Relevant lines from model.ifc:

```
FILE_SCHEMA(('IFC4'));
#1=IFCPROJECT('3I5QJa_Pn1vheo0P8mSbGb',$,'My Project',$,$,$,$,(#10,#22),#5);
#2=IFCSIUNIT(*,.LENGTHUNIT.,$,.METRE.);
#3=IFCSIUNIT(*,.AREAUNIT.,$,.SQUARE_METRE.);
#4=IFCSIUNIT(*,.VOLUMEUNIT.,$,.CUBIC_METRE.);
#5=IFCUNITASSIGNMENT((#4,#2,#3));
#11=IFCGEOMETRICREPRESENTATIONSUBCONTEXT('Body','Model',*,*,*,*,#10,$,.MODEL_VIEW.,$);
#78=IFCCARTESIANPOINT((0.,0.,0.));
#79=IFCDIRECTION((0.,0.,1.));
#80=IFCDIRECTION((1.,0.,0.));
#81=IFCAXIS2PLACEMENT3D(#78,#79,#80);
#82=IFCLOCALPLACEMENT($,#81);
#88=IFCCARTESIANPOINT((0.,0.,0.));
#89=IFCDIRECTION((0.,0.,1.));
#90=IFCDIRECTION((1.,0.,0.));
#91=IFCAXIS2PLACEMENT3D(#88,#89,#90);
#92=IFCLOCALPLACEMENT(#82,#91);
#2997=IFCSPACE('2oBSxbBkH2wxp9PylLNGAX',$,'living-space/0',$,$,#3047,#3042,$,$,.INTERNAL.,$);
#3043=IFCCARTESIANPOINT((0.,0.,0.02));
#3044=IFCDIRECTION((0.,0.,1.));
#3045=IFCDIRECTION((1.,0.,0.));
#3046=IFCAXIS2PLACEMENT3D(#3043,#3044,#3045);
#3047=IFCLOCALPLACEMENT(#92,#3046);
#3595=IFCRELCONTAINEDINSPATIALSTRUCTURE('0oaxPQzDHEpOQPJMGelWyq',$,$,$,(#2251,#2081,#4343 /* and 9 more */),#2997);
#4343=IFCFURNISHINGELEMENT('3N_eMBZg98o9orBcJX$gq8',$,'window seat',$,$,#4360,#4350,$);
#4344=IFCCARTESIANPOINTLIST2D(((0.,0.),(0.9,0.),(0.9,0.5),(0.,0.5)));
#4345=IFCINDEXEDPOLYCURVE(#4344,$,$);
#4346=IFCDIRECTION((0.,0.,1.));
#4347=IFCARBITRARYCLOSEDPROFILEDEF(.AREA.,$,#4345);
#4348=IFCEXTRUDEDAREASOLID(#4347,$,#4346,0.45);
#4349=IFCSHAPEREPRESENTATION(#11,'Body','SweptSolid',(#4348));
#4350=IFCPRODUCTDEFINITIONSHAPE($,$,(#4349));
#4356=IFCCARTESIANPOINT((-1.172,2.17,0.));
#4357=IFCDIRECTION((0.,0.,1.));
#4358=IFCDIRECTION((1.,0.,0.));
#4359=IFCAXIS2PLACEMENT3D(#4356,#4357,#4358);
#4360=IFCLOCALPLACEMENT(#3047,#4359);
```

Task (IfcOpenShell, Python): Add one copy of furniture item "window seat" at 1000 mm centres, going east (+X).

```python
import numpy as np
import ifcopenshell
import ifcopenshell.api.geometry
import ifcopenshell.api.root
import ifcopenshell.util.element
import ifcopenshell.util.placement
import ifcopenshell.util.unit

model = ifcopenshell.open("model.ifc")
unit_scale = ifcopenshell.util.unit.calculate_unit_scale(model)

source = model.by_id(4343)
base = ifcopenshell.util.placement.get_local_placement(source.ObjectPlacement)
step = np.array([1.0, 0.0, 0.0]) * 1 / unit_scale

for i in range(1, 2):
    copy = ifcopenshell.api.root.copy_class(model, product=source)
    copy.Representation = ifcopenshell.util.element.copy_deep(
        model, source.Representation, exclude=["IfcGeometricRepresentationContext", "IfcRepresentationMap"]
    )
    matrix = base.copy()
    matrix[:3, 3] += i * step
    print("added at", matrix[:3, 3].round(3) + 0.0)
    ifcopenshell.api.geometry.edit_object_placement(model, product=copy, matrix=matrix, is_si=False)

model.write("model_edited.ifc")
```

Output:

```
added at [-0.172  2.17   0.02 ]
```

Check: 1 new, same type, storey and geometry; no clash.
